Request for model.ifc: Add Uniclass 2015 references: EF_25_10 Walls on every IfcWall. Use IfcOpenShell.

First a look at what the model holds.

```python
import ifcopenshell

model = ifcopenshell.open("model.ifc")
print(model.schema)
print("classifications:", [c.Name for c in model.by_type("IfcClassification")])
for ifc_class in ("IfcDoor", "IfcRoof", "IfcStair", "IfcWall", "IfcWindow"):
    print(ifc_class, len(model.by_type(ifc_class)))
```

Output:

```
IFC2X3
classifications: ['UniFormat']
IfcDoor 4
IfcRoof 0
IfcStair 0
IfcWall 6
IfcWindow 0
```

```python
import ifcopenshell
import ifcopenshell.api.classification

model = ifcopenshell.open("model.ifc")

# IFC2X3 requires Source and Edition and has no link from the project to the system.
system = model.create_entity("IfcClassification", Source="NBS", Edition="2015", Name="Uniclass 2015")

codes = {
    "IfcWall": ("EF_25_10", "Walls"),
}
for ifc_class, (code, name) in codes.items():
    products = model.by_type(ifc_class)
    ifcopenshell.api.classification.add_reference(
        model, products=products, classification=system, identification=code, name=name
    )
    print(code, len(products))

model.write("model_v2.ifc")
```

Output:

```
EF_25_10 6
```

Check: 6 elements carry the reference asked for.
